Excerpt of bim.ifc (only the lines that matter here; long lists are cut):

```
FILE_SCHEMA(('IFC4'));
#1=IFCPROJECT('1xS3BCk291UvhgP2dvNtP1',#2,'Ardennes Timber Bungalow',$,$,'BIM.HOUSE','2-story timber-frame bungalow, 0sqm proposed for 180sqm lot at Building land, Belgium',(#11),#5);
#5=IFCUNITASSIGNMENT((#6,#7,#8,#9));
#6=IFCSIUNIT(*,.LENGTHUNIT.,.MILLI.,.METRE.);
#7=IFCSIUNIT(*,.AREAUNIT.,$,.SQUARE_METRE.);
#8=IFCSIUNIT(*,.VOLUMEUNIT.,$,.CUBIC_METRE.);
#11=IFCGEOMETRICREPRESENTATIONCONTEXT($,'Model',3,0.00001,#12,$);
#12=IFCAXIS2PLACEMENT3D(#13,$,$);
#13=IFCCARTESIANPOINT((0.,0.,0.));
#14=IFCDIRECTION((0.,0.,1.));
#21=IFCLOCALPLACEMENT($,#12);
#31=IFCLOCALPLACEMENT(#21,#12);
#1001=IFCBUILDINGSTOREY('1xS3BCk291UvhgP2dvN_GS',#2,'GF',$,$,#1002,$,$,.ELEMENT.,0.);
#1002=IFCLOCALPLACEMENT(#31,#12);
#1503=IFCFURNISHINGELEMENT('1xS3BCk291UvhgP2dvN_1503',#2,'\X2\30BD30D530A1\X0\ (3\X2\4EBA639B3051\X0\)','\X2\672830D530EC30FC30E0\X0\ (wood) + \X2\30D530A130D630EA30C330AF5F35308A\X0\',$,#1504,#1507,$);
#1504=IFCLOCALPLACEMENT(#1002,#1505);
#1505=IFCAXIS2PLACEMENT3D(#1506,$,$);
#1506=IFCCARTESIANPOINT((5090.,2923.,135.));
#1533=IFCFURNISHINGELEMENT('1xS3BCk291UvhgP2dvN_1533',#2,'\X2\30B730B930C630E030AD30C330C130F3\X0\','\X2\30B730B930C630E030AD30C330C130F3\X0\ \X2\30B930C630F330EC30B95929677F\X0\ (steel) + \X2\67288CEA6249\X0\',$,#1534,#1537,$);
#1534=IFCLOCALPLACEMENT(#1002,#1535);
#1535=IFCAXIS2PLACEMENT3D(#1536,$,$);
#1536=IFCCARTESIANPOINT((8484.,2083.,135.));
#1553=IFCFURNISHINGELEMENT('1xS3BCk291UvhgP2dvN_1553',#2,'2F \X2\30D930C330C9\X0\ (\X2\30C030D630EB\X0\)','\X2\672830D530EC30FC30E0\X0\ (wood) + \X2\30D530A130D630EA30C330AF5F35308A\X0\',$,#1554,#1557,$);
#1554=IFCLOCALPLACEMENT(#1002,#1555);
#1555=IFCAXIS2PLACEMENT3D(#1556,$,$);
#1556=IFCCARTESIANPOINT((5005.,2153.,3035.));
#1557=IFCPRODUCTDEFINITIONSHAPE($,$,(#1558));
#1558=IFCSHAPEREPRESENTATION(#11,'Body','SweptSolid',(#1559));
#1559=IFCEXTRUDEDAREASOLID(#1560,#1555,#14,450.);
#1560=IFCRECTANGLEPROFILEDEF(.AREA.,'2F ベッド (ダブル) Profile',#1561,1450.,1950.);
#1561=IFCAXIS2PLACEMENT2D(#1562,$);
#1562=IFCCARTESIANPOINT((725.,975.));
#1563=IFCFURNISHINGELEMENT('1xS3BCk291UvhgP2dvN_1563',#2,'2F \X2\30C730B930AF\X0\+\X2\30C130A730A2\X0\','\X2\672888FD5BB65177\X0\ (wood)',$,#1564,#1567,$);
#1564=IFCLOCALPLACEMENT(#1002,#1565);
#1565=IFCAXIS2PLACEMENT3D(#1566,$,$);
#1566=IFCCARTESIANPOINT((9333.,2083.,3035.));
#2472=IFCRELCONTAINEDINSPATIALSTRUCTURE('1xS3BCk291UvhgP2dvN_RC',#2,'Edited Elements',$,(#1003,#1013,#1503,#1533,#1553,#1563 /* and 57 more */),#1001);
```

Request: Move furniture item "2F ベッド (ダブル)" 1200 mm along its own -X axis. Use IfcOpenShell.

```python
import ifcopenshell
import ifcopenshell.api.geometry
import ifcopenshell.util.placement

model = ifcopenshell.open("bim.ifc")

item = model.by_id(1553)
matrix = ifcopenshell.util.placement.get_local_placement(item.ObjectPlacement)
matrix[:3, 3] -= matrix[:3, 0] * 1200.0
ifcopenshell.api.geometry.edit_object_placement(model, product=item, matrix=matrix, is_si=False)

print(ifcopenshell.util.placement.get_local_placement(item.ObjectPlacement).round(3) + 0.0)

model.write("bim_edited.ifc")
```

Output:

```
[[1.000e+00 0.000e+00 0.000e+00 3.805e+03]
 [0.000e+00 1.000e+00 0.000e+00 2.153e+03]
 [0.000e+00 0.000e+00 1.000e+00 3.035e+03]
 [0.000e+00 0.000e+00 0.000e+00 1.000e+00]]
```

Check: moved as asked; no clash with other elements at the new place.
